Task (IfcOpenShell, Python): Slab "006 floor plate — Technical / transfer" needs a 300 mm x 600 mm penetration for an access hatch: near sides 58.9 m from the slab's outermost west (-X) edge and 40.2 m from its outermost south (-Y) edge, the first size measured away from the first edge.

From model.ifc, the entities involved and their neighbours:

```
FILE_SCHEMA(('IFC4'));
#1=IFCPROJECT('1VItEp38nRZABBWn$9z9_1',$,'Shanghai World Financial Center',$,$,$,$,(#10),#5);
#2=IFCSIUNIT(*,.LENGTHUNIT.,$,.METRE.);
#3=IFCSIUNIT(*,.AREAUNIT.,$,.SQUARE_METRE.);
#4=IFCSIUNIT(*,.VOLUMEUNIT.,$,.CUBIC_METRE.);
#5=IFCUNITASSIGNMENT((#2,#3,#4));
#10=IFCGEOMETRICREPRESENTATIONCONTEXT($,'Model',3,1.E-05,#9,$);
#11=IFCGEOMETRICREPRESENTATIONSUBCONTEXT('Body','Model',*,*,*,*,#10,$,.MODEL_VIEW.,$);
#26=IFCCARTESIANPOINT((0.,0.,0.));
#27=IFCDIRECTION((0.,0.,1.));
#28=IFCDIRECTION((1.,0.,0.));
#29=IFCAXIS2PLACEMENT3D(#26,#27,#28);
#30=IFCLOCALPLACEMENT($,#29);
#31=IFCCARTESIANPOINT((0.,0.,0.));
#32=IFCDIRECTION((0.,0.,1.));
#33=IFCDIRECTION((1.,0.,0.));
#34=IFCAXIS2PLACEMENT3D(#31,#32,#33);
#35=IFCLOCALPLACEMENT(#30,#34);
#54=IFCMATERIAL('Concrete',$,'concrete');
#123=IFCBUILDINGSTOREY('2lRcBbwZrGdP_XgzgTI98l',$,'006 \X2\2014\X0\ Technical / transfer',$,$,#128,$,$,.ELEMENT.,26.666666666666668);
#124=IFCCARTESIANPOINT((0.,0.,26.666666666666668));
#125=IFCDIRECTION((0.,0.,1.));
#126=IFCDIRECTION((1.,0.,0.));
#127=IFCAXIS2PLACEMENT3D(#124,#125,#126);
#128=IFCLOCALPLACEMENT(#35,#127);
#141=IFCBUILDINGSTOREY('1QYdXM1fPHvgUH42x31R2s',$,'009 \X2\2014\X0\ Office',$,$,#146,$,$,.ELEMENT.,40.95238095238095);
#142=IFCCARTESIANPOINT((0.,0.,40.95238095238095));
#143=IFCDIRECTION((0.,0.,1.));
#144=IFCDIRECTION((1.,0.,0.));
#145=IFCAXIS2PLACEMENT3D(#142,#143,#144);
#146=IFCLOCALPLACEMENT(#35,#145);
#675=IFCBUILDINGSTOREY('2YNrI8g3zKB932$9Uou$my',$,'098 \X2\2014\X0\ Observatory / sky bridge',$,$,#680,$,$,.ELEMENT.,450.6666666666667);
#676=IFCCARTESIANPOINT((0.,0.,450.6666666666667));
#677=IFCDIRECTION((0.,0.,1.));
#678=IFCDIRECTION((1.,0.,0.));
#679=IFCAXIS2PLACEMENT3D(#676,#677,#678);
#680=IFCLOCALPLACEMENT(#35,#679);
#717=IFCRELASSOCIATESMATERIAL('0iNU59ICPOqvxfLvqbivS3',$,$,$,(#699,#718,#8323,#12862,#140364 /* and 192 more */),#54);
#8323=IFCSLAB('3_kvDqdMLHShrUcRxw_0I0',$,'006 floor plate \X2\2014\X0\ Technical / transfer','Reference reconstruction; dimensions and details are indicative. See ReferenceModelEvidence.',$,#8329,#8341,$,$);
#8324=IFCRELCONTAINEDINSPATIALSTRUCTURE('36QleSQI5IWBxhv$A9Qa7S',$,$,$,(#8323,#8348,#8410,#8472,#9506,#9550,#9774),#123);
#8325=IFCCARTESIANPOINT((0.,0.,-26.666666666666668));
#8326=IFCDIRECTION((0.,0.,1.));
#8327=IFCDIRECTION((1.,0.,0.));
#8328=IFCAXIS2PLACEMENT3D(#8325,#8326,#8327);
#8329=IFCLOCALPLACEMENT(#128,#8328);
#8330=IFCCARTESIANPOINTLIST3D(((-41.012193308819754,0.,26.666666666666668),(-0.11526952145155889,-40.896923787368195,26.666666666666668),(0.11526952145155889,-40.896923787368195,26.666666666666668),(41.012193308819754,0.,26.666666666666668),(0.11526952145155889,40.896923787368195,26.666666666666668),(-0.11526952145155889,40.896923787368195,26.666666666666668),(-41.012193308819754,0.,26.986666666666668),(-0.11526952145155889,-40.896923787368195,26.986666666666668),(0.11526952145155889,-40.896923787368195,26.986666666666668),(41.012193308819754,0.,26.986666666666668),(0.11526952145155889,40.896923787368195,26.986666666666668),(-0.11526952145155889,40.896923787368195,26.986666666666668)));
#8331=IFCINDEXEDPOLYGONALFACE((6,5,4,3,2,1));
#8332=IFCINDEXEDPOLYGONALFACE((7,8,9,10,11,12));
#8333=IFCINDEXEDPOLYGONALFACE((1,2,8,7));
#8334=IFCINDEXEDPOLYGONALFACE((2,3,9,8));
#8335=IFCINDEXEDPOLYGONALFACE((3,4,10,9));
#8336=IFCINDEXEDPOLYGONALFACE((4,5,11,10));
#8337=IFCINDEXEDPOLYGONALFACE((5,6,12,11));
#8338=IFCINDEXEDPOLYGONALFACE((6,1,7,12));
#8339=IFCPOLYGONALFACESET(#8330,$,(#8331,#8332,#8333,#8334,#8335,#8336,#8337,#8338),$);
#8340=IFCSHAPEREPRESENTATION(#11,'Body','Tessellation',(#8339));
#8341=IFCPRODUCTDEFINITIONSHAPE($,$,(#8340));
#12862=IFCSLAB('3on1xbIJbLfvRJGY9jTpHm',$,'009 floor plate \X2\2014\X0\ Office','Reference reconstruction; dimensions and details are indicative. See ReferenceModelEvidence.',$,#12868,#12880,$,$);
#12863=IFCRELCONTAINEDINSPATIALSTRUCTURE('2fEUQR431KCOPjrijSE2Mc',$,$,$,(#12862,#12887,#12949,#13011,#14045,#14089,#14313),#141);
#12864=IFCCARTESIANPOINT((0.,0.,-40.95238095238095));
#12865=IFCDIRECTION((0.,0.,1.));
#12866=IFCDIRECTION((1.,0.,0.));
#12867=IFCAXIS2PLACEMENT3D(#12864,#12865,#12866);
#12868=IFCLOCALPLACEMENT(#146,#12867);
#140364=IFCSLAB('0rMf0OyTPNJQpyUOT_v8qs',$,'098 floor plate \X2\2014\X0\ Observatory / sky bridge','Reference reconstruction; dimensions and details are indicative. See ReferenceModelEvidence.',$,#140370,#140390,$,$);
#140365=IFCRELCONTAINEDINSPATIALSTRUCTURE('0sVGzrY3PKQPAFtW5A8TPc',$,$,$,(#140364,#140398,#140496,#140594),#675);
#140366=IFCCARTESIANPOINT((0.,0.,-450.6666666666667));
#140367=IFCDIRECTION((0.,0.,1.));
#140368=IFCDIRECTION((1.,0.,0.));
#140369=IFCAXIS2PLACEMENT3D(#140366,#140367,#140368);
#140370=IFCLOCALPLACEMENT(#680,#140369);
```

```python
import numpy as np
import ifcopenshell
import ifcopenshell.api.feature
import ifcopenshell.api.geometry
import ifcopenshell.api.root
import ifcopenshell.geom
import ifcopenshell.util.placement
import ifcopenshell.util.representation
import ifcopenshell.util.shape
import ifcopenshell.util.unit

model = ifcopenshell.open("model.ifc")
unit_scale = ifcopenshell.util.unit.calculate_unit_scale(model)
settings = ifcopenshell.geom.settings()


def volume(element):
    """Net volume in cubic metres, openings subtracted."""
    shape = ifcopenshell.geom.create_shape(settings, element)
    return ifcopenshell.util.shape.get_volume(shape.geometry)


slab = model.by_id(8323)
before = volume(slab)

# Extent in the slab's own axes, in metres. The edges named are its -X and -Y sides.
slab_shape = ifcopenshell.geom.create_shape(settings, slab)
vertices = ifcopenshell.util.shape.get_vertices(slab_shape.geometry)
x_min, y_min, bottom = vertices.min(axis=0)
top = vertices[:, 2].max()

opening = ifcopenshell.api.root.create_entity(model, ifc_class="IfcOpeningElement", name="Access hatch opening", predefined_type="OPENING")
context = ifcopenshell.util.representation.get_context(model, "Model", "Body", "MODEL_VIEW")
width, depth = 0.3, 0.6
outline = [(0.0, 0.0), (width, 0.0), (width, depth), (0.0, depth), (0.0, 0.0)]
# Overshoot both faces by 50 mm so the cut is clean.
shape = ifcopenshell.api.geometry.add_slab_representation(
    model, context=context, depth=top - bottom + 0.1, polyline=outline
)
ifcopenshell.api.geometry.assign_representation(model, product=opening, representation=shape)

matrix = ifcopenshell.util.placement.get_local_placement(slab.ObjectPlacement)
matrix[:, 3] = matrix @ np.append(np.array([x_min + 58.9, y_min + 40.2, bottom - 0.05]) / unit_scale, 1.0)
ifcopenshell.api.geometry.edit_object_placement(model, product=opening, matrix=matrix, is_si=False)
ifcopenshell.api.feature.add_feature(model, feature=opening, element=slab)

after = volume(slab)

print(f"slab volume {before:.3f} -> {after:.3f} m3")

model.write("model-out.ifc")
```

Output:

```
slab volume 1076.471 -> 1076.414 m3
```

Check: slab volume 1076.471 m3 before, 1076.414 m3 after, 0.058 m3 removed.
